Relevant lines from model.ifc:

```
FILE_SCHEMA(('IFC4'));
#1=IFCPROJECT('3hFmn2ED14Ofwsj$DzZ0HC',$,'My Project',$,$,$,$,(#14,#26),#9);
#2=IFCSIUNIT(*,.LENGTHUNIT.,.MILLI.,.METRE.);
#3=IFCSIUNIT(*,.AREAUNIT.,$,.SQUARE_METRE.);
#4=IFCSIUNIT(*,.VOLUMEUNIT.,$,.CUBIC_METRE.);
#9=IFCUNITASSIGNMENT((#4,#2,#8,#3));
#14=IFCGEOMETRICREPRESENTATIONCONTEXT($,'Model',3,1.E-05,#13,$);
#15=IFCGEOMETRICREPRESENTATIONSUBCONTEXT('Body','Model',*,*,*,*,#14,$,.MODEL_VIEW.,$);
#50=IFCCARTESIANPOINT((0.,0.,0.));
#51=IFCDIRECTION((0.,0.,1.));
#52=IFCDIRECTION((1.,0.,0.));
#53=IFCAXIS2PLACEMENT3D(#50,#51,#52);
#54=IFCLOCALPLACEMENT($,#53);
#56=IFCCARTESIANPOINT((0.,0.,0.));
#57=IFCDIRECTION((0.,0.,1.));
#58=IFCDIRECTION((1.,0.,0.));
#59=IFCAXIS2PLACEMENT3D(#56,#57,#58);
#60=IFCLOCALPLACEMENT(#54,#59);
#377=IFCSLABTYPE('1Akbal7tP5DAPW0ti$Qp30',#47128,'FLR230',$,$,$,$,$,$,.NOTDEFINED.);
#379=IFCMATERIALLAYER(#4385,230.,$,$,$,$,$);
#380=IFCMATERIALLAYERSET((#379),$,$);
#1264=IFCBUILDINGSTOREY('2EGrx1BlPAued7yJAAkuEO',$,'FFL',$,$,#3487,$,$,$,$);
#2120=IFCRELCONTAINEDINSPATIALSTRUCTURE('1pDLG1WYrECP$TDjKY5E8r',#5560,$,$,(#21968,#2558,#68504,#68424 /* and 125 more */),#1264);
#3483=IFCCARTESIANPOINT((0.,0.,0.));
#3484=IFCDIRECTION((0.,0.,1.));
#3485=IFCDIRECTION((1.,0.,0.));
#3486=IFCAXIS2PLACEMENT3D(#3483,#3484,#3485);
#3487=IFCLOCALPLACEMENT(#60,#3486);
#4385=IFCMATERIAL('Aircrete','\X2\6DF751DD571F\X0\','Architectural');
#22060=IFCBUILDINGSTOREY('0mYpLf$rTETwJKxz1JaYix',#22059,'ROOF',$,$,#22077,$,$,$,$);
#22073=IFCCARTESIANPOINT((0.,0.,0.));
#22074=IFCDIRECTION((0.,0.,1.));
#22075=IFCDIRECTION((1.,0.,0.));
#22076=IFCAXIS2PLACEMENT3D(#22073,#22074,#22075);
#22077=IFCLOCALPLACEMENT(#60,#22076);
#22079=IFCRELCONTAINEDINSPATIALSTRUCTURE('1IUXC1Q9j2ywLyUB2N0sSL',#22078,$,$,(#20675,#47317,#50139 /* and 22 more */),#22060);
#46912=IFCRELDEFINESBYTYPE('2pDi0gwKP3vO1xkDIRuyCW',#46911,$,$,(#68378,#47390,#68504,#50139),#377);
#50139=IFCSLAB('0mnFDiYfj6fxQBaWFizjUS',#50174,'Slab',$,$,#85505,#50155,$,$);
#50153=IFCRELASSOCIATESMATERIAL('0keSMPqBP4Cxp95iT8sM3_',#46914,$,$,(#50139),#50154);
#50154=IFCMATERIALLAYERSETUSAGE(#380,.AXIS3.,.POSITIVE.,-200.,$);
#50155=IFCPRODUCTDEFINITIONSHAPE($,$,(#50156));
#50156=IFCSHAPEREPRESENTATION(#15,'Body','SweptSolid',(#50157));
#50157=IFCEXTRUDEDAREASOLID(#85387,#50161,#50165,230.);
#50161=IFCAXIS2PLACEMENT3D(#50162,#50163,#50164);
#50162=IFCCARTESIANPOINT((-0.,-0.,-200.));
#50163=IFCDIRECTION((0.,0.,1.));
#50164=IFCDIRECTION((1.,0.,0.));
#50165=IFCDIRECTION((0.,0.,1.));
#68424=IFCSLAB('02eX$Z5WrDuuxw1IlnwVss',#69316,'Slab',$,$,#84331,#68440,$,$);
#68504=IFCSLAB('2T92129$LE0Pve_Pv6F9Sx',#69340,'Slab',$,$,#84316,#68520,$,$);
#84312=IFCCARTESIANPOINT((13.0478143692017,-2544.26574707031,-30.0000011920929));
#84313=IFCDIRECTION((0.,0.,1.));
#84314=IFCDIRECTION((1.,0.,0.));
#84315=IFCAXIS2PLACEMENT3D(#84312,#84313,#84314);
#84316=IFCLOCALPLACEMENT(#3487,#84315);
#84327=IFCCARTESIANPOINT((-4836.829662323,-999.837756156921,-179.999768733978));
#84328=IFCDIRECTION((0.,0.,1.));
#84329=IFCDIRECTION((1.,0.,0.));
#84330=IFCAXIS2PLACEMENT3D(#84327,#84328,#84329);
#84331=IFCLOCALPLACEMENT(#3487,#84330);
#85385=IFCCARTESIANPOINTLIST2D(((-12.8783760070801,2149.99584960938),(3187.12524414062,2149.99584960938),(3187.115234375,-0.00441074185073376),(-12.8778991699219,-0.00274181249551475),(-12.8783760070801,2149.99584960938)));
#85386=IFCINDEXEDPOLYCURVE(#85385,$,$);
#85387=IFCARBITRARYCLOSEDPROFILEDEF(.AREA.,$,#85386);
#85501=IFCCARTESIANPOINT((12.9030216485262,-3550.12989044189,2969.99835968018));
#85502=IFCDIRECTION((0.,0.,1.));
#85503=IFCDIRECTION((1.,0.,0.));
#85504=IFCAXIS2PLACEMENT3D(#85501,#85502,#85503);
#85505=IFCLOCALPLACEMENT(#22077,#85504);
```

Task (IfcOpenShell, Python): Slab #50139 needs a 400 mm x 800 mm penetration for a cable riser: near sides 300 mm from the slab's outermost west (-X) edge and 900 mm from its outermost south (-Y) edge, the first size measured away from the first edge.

```python
import numpy as np
import ifcopenshell
import ifcopenshell.api.feature
import ifcopenshell.api.geometry
import ifcopenshell.api.root
import ifcopenshell.geom
import ifcopenshell.util.placement
import ifcopenshell.util.representation
import ifcopenshell.util.shape
import ifcopenshell.util.unit

model = ifcopenshell.open("model.ifc")
unit_scale = ifcopenshell.util.unit.calculate_unit_scale(model)
settings = ifcopenshell.geom.settings()


def volume(element):
    """Net volume in cubic metres, openings subtracted."""
    shape = ifcopenshell.geom.create_shape(settings, element)
    return ifcopenshell.util.shape.get_volume(shape.geometry)


slab = model.by_guid("0mnFDiYfj6fxQBaWFizjUS")
before = volume(slab)

# Extent in the slab's own axes, in metres. The edges named are its -X and -Y sides.
slab_shape = ifcopenshell.geom.create_shape(settings, slab)
vertices = ifcopenshell.util.shape.get_vertices(slab_shape.geometry)
x_min, y_min, bottom = vertices.min(axis=0)
top = vertices[:, 2].max()

opening = ifcopenshell.api.root.create_entity(model, ifc_class="IfcOpeningElement", name="Cable riser opening", predefined_type="OPENING")
context = ifcopenshell.util.representation.get_context(model, "Model", "Body", "MODEL_VIEW")
width, depth = 0.4, 0.8
outline = [(0.0, 0.0), (width, 0.0), (width, depth), (0.0, depth), (0.0, 0.0)]
# Overshoot both faces by 50 mm so the cut is clean.
shape = ifcopenshell.api.geometry.add_slab_representation(
    model, context=context, depth=top - bottom + 0.1, polyline=outline
)
ifcopenshell.api.geometry.assign_representation(model, product=opening, representation=shape)

matrix = ifcopenshell.util.placement.get_local_placement(slab.ObjectPlacement)
matrix[:, 3] = matrix @ np.append(np.array([x_min + 0.3, y_min + 0.9, bottom - 0.05]) / unit_scale, 1.0)
ifcopenshell.api.geometry.edit_object_placement(model, product=opening, matrix=matrix, is_si=False)
ifcopenshell.api.feature.add_feature(model, feature=opening, element=slab)

after = volume(slab)

print(f"slab volume {before:.3f} -> {after:.3f} m3")

model.write("model_rev.ifc")
```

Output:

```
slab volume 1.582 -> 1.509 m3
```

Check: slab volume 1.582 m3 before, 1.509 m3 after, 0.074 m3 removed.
